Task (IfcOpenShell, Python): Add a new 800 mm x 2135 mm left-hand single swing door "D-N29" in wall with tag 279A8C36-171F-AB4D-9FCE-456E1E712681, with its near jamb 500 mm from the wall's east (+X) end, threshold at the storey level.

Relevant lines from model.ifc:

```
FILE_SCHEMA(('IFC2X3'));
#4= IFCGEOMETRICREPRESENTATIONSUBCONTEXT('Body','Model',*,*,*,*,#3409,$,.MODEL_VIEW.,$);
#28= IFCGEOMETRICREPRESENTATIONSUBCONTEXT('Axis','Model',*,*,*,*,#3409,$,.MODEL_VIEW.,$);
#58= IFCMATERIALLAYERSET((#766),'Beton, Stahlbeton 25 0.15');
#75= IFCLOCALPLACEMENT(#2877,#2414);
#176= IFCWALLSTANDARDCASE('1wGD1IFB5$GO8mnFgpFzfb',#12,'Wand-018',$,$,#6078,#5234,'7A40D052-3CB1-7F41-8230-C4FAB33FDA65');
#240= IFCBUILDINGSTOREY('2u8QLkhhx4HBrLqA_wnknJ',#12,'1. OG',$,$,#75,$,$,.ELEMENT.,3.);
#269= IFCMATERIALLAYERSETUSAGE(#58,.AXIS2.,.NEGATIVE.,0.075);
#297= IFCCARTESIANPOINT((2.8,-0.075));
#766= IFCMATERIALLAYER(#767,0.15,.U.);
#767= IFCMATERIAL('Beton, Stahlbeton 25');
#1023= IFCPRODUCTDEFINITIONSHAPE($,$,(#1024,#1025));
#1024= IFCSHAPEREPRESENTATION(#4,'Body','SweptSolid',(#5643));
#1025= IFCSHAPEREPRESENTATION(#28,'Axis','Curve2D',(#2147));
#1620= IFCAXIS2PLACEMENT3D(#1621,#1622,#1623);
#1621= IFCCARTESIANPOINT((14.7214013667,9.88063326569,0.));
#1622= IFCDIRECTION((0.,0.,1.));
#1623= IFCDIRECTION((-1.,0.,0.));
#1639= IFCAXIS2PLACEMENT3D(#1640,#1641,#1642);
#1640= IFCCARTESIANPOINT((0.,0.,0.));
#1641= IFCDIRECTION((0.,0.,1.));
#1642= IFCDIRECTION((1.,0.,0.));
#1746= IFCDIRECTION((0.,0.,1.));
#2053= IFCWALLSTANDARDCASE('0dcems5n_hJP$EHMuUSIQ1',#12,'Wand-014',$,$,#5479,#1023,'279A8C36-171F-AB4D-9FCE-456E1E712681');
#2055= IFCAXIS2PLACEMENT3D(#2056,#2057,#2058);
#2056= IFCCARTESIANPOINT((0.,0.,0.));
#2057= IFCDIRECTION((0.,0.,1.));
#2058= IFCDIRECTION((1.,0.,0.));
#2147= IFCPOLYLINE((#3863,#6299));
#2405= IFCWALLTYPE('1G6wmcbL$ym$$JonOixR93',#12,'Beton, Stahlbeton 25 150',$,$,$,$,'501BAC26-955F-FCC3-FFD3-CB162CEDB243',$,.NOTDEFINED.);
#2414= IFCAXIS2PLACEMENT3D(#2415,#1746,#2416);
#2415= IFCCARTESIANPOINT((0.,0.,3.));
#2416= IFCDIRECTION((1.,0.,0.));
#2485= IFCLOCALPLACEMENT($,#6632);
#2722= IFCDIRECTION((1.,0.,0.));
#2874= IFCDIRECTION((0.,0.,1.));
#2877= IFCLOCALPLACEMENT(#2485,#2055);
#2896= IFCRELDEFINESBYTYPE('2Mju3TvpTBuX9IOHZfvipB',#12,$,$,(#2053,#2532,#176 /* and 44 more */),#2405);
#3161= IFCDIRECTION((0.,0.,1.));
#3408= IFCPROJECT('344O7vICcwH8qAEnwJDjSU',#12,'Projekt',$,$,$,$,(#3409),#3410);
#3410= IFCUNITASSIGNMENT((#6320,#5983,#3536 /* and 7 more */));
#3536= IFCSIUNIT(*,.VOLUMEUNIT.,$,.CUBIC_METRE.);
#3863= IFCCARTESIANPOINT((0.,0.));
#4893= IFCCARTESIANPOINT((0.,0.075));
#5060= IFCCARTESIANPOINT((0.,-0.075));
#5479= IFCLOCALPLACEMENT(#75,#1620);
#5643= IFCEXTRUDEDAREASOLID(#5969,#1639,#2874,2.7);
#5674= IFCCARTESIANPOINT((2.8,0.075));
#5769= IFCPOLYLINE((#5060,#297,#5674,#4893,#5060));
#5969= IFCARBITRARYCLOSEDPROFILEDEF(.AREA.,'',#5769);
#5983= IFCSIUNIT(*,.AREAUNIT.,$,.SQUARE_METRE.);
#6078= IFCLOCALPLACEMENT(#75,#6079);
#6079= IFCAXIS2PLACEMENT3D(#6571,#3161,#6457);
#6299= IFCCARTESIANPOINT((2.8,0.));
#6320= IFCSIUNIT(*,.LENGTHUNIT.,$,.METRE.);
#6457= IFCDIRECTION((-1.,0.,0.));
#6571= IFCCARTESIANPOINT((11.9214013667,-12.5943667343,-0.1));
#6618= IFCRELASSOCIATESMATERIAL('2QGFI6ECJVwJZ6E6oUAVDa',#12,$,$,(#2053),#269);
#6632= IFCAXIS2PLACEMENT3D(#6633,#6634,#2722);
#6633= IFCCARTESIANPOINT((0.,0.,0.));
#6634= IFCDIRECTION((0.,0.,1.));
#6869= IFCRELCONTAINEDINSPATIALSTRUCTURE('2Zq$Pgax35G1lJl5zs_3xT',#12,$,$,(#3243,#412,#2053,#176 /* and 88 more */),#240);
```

```python
import numpy as np
import ifcopenshell
import ifcopenshell.api.feature
import ifcopenshell.api.geometry
import ifcopenshell.api.root
import ifcopenshell.api.spatial
import ifcopenshell.api.type
import ifcopenshell.geom
import ifcopenshell.util.element
import ifcopenshell.util.placement
import ifcopenshell.util.representation
import ifcopenshell.util.shape
import ifcopenshell.util.unit

model = ifcopenshell.open("model.ifc")
unit_scale = ifcopenshell.util.unit.calculate_unit_scale(model)
settings = ifcopenshell.geom.settings()


def volume(element):
    """Net volume in cubic metres, openings subtracted."""
    shape = ifcopenshell.geom.create_shape(settings, element)
    return ifcopenshell.util.shape.get_volume(shape.geometry)


wall = model.by_id(2053)
storey = ifcopenshell.util.element.get_container(wall, ifc_class="IfcBuildingStorey")
context = ifcopenshell.util.representation.get_context(model, "Model", "Body", "MODEL_VIEW")
before = volume(wall)

width, height, from_end, sill = 0.8, 2.135, 0.5, 0.0  # metres

# The wall runs along its own X axis, and the end named is its -X end.
wall_shape = ifcopenshell.geom.create_shape(settings, wall)
x, y, z = ifcopenshell.util.shape.get_vertices(wall_shape.geometry).T
start = x.min() + from_end
face, thickness = float(y.min()), float(y.max() - y.min())
wall_matrix = ifcopenshell.util.placement.get_local_placement(wall.ObjectPlacement)
level = ifcopenshell.util.placement.get_local_placement(storey.ObjectPlacement)[2, 3]


def in_wall(x, y):
    """Placement at x, y metres in the wall's axes, at sill height."""
    matrix = wall_matrix.copy()
    matrix[:, 3] = wall_matrix @ np.array([x / unit_scale, y / unit_scale, 0.0, 1.0])
    matrix[2, 3] = level + sill / unit_scale
    return matrix


# Opening: a box that overshoots both wall faces by 50 mm.
opening = ifcopenshell.api.root.create_entity(model, ifc_class="IfcOpeningElement")
box = ifcopenshell.api.geometry.add_wall_representation(
    model, context=context, length=width, height=height, thickness=thickness + 0.1
)
ifcopenshell.api.geometry.assign_representation(model, product=opening, representation=box)
ifcopenshell.api.geometry.edit_object_placement(model, product=opening, matrix=in_wall(start, face - 0.05), is_si=False)
ifcopenshell.api.feature.add_feature(model, feature=opening, element=wall)

door = ifcopenshell.api.root.create_entity(model, ifc_class="IfcDoor", name="D-N29")
door.OverallWidth, door.OverallHeight = width / unit_scale, height / unit_scale
body = ifcopenshell.api.geometry.add_door_representation(
    model,
    context=context,
    overall_width=door.OverallWidth,
    overall_height=door.OverallHeight,
    operation_type="SINGLE_SWING_LEFT",
    lining_properties={"LiningDepth": thickness / unit_scale, "ThresholdDepth": thickness / unit_scale},
)
ifcopenshell.api.geometry.assign_representation(model, product=door, representation=body)
ifcopenshell.api.spatial.assign_container(model, products=[door], relating_structure=storey)
fills = ifcopenshell.api.feature.add_filling(model, opening=opening, element=door)
fills.OwnerHistory = door.OwnerHistory  # required in IFC2X3

# IFC2X3 keeps the operation on the door style.
style = ifcopenshell.api.root.create_entity(model, ifc_class="IfcDoorStyle", name="D-N29")
style.OperationType, style.ConstructionType = "SINGLE_SWING_LEFT", "NOTDEFINED"
style.ParameterTakesPrecedence = style.Sizeable = False
ifcopenshell.api.type.assign_type(model, related_objects=[door], relating_type=style)

# The lining spans the wall, so the door starts at the wall face.
ifcopenshell.api.geometry.edit_object_placement(model, product=door, matrix=in_wall(start, face), is_si=False)

after = volume(wall)

print(f"wall volume {before:.3f} -> {after:.3f} m3")

model.write("model_updated.ifc")
```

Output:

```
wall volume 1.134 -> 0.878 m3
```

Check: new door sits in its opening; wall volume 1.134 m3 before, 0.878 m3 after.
